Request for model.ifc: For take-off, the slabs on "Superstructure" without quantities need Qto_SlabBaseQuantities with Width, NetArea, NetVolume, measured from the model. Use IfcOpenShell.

First a look at what the model holds.

```python
import ifcopenshell
import ifcopenshell.util.element
import ifcopenshell.util.unit

model = ifcopenshell.open("model.ifc")
print(model.schema)
for unit_type in ("LENGTHUNIT", "AREAUNIT", "VOLUMEUNIT"):
    print(unit_type, ifcopenshell.util.unit.calculate_unit_scale(model, unit_type))
storey = next(s for s in model.by_type("IfcBuildingStorey") if s.Name == "Superstructure")
slabs = [e for e in ifcopenshell.util.element.get_decomposition(storey) if e.is_a("IfcSlab")]
for e in sorted(slabs, key=lambda e: e.id()):
    print(e.id(), e.is_a(), e.Name, list(ifcopenshell.util.element.get_psets(e, qtos_only=True)), sep=" | ")
```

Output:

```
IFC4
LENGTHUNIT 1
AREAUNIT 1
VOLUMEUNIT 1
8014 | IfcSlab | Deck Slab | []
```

```python
import ifcopenshell
import ifcopenshell.api.pset
import ifcopenshell.geom
import ifcopenshell.util.element
import ifcopenshell.util.shape
import ifcopenshell.util.unit

model = ifcopenshell.open("model.ifc")
unit_scale = ifcopenshell.util.unit.calculate_unit_scale(model)
area_scale = ifcopenshell.util.unit.calculate_unit_scale(model, "AREAUNIT")
volume_scale = ifcopenshell.util.unit.calculate_unit_scale(model, "VOLUMEUNIT")
settings = ifcopenshell.geom.settings()

storey = next(s for s in model.by_type("IfcBuildingStorey") if s.Name == "Superstructure")
slabs = [e for e in ifcopenshell.util.element.get_decomposition(storey) if e.is_a("IfcSlab")]

for e in sorted(slabs, key=lambda e: e.id()):
    if ifcopenshell.util.element.get_psets(e, qtos_only=True, should_inherit=False):
        continue
    # Geometry comes back in metres, in the element's own axes.
    shape = ifcopenshell.geom.create_shape(settings, e)
    values = {
        "Width": ifcopenshell.util.shape.get_z(shape.geometry) / unit_scale,
        "NetArea": ifcopenshell.util.shape.get_footprint_area(shape.geometry) / area_scale,
        "NetVolume": ifcopenshell.util.shape.get_volume(shape.geometry) / volume_scale,
    }
    qto = ifcopenshell.api.pset.add_qto(model, product=e, name="Qto_SlabBaseQuantities")
    ifcopenshell.api.pset.edit_qto(model, qto=qto, properties=values)
    print(e.id(), {k: round(v, 3) for k, v in values.items()})

model.write("model_edited.ifc")
```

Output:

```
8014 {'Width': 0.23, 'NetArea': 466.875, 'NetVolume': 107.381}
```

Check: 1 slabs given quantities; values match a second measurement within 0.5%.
